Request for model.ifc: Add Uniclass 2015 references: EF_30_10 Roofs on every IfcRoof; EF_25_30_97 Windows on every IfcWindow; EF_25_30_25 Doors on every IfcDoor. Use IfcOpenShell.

First a look at what the model holds.

```python
import ifcopenshell

model = ifcopenshell.open("model.ifc")
print(model.schema)
print("classifications:", [c.Name for c in model.by_type("IfcClassification")])
for ifc_class in ("IfcDoor", "IfcRoof", "IfcStair", "IfcWall", "IfcWindow"):
    print(ifc_class, len(model.by_type(ifc_class)))
```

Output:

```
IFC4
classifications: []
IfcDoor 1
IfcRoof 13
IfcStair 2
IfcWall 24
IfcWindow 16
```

```python
import ifcopenshell
import ifcopenshell.api.classification

model = ifcopenshell.open("model.ifc")

system = ifcopenshell.api.classification.add_classification(model, classification="Uniclass 2015")

codes = {
    "IfcRoof": ("EF_30_10", "Roofs"),
    "IfcWindow": ("EF_25_30_97", "Windows"),
    "IfcDoor": ("EF_25_30_25", "Doors"),
}
for ifc_class, (code, name) in codes.items():
    products = model.by_type(ifc_class)
    ifcopenshell.api.classification.add_reference(
        model, products=products, classification=system, identification=code, name=name
    )
    print(code, len(products))

model.write("model-out.ifc")
```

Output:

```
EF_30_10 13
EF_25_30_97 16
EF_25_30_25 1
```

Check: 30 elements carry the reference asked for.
